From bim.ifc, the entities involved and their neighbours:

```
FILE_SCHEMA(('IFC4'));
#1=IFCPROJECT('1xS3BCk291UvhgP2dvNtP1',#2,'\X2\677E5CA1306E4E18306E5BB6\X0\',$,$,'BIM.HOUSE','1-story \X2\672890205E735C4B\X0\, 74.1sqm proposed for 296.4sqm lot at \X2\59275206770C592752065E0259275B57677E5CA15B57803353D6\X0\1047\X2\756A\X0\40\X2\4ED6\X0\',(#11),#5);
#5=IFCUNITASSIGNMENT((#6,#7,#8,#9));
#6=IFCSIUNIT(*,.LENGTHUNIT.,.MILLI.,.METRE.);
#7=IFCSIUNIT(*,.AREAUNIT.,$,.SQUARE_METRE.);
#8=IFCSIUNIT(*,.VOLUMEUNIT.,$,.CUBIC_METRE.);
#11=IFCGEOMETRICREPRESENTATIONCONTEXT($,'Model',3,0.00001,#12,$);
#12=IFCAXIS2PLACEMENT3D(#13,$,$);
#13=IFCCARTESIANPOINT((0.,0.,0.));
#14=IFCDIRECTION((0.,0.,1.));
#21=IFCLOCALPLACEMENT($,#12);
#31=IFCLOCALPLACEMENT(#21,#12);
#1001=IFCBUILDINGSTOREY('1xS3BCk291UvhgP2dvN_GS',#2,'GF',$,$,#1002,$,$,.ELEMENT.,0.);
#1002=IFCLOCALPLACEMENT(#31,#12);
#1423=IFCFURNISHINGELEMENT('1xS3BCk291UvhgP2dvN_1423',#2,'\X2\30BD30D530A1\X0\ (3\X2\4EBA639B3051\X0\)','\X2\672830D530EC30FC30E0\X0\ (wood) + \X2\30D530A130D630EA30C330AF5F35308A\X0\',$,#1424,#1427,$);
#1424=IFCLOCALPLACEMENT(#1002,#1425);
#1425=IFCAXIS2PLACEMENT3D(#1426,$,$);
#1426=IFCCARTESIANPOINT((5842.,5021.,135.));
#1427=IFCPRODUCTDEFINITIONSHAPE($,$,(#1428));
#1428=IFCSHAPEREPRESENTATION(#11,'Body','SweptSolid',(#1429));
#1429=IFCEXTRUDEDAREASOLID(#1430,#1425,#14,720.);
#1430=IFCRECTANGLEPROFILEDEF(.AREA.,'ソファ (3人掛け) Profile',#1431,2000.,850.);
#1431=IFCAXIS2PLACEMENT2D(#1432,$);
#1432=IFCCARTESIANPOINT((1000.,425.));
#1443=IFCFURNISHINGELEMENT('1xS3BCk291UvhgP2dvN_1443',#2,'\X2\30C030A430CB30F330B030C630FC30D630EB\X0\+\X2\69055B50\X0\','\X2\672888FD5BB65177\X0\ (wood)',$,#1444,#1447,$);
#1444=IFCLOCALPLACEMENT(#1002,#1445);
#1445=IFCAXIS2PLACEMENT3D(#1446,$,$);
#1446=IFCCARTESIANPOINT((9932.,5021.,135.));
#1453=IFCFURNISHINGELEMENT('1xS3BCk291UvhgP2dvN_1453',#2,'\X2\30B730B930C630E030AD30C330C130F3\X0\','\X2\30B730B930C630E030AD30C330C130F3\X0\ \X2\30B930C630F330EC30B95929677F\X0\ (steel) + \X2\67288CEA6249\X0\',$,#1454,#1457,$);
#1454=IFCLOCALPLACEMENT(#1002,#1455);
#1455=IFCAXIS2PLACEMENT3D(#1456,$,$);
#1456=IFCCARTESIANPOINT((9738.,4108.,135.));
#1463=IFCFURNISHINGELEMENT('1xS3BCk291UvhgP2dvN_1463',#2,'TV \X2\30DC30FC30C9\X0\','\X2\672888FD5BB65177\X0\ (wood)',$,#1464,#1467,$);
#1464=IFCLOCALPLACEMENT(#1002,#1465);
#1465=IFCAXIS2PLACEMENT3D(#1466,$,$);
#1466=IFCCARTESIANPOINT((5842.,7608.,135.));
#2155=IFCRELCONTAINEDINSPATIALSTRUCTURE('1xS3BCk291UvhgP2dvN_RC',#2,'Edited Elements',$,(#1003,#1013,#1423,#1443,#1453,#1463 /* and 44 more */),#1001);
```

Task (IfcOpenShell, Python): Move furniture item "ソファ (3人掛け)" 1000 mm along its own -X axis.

```python
import ifcopenshell
import ifcopenshell.api.geometry
import ifcopenshell.util.placement

model = ifcopenshell.open("bim.ifc")

item = model.by_id(1423)
matrix = ifcopenshell.util.placement.get_local_placement(item.ObjectPlacement)
matrix[:3, 3] -= matrix[:3, 0] * 1000.0
ifcopenshell.api.geometry.edit_object_placement(model, product=item, matrix=matrix, is_si=False)

print(ifcopenshell.util.placement.get_local_placement(item.ObjectPlacement).round(3) + 0.0)

model.write("bim-out.ifc")
```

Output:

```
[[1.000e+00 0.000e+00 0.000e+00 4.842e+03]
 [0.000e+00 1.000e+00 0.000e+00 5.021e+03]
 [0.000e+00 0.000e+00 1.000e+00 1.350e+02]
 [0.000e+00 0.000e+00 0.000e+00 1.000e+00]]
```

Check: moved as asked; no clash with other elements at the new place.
